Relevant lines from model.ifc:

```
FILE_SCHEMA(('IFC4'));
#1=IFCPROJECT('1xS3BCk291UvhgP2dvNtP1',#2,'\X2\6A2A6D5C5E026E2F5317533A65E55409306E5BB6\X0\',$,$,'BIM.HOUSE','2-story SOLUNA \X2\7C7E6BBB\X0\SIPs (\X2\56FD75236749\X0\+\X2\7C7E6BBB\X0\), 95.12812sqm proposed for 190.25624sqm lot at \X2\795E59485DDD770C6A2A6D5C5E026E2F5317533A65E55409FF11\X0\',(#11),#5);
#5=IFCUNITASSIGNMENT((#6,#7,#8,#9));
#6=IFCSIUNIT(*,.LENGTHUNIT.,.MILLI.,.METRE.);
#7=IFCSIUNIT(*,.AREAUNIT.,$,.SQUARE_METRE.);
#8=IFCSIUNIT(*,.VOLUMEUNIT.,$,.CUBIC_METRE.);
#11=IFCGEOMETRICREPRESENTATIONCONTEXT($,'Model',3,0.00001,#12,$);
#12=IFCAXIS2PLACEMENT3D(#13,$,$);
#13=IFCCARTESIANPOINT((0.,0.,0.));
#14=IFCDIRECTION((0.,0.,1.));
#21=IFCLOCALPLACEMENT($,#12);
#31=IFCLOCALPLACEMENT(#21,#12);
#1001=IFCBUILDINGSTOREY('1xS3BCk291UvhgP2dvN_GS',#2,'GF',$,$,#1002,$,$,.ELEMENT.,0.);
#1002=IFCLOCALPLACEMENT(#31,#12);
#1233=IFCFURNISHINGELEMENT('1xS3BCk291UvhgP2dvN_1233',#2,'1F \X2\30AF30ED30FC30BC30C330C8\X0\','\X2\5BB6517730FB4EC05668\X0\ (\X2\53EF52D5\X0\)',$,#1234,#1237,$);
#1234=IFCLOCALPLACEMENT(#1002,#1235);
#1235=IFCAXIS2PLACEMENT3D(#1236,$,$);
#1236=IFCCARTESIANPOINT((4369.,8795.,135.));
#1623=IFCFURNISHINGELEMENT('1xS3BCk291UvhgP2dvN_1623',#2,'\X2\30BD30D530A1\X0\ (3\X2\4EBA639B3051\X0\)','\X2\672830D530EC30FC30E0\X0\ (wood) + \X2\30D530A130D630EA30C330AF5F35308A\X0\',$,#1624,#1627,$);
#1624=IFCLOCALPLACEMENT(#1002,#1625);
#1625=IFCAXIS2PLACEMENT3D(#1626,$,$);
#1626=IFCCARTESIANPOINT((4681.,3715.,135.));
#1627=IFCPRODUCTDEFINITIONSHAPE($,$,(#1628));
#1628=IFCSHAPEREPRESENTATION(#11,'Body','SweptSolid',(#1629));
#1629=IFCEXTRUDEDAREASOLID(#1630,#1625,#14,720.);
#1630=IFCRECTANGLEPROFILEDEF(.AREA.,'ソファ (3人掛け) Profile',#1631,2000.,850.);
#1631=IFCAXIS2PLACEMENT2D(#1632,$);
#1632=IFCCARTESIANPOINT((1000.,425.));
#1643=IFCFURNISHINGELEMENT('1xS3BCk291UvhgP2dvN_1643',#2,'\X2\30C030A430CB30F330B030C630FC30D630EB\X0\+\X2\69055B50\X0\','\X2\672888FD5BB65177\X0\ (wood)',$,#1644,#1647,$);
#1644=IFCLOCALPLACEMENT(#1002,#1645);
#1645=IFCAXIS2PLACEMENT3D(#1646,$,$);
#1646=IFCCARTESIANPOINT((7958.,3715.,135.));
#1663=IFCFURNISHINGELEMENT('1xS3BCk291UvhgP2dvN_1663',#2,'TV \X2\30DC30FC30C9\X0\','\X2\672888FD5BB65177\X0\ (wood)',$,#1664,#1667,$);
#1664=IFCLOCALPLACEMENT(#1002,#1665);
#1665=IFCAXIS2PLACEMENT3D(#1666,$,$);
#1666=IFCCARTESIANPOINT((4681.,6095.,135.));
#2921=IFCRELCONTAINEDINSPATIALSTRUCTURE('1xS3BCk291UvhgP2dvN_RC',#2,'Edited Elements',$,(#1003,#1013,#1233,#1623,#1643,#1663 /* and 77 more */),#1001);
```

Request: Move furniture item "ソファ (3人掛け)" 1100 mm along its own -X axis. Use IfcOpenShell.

```python
import ifcopenshell
import ifcopenshell.api.geometry
import ifcopenshell.util.placement

model = ifcopenshell.open("model.ifc")

item = model.by_id(1623)
matrix = ifcopenshell.util.placement.get_local_placement(item.ObjectPlacement)
matrix[:3, 3] -= matrix[:3, 0] * 1100.0
ifcopenshell.api.geometry.edit_object_placement(model, product=item, matrix=matrix, is_si=False)

print(ifcopenshell.util.placement.get_local_placement(item.ObjectPlacement).round(3) + 0.0)

model.write("model_edited.ifc")
```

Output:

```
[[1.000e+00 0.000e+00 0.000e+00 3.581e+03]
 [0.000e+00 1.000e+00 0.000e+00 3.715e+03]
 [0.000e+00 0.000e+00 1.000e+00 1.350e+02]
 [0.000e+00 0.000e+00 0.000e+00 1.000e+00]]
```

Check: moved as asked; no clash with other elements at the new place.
